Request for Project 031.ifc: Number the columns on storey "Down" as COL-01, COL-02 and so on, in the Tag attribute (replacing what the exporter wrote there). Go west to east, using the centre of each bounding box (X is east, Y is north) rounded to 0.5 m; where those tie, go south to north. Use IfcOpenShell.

First a look at what the model holds.

```python
import ifcopenshell
import ifcopenshell.util.element
import ifcopenshell.util.placement

model = ifcopenshell.open("Project 031.ifc")
print(model.schema)
storey = next(s for s in model.by_type("IfcBuildingStorey") if s.Name == "Down")
columns = [e for e in ifcopenshell.util.element.get_decomposition(storey) if e.is_a("IfcColumn")]
for e in sorted(columns, key=lambda e: e.id()):
    origin = ifcopenshell.util.placement.get_local_placement(e.ObjectPlacement)[:3, 3]
    print(e.id(), e.Tag, e.Name, origin.round(2) + 0.0, sep=" | ")
```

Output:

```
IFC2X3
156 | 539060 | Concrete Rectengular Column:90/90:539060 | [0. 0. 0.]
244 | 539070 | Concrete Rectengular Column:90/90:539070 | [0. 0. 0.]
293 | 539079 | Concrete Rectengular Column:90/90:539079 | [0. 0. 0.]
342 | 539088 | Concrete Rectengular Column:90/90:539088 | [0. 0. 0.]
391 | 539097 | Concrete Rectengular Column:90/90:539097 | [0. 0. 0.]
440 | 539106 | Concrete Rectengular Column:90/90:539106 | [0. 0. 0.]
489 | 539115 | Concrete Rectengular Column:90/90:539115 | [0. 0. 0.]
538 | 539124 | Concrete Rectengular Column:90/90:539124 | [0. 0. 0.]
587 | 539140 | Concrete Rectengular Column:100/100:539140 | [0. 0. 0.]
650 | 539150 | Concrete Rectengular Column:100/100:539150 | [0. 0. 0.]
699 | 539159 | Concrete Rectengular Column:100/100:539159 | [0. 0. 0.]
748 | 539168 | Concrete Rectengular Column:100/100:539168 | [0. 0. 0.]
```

```python
import ifcopenshell
import ifcopenshell.geom
import ifcopenshell.util.element
import ifcopenshell.util.shape

model = ifcopenshell.open("Project 031.ifc")
settings = ifcopenshell.geom.settings()
settings.set("use-world-coords", True)


def centre(element):
    shape = ifcopenshell.geom.create_shape(settings, element)
    return ifcopenshell.util.shape.get_bbox_centroid(shape.geometry)


storey = next(s for s in model.by_type("IfcBuildingStorey") if s.Name == "Down")
columns = [e for e in ifcopenshell.util.element.get_decomposition(storey) if e.is_a("IfcColumn")]

# Insertion points can sit at a corner or the storey origin, so sort by the geometry (in metres).
centres = {e: centre(e) for e in columns}
columns.sort(key=lambda e: (round(centres[e][0] / 0.5), centres[e][1]))

for i, e in enumerate(columns, start=1):
    number = f"COL-{i:02d}"
    e.Tag = number
    print(e.id(), number)

model.write("Project 031_v2.ifc")
```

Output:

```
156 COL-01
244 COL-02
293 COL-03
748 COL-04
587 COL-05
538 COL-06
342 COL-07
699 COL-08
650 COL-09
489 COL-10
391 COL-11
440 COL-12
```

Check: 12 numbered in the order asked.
